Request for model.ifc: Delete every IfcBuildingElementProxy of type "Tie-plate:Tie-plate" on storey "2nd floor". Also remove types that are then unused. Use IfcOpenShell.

First a look at what the model holds.

```python
import ifcopenshell
import ifcopenshell.util.element

model = ifcopenshell.open("model.ifc")
print(model.schema)
storey = next(s for s in model.by_type("IfcBuildingStorey") if s.Name == "2nd floor")
proxies = [e for e in ifcopenshell.util.element.get_decomposition(storey) if e.is_a("IfcBuildingElementProxy")]
seen = {}
for e in proxies:
    element_type = ifcopenshell.util.element.get_type(e)
    name = element_type.Name if element_type not in (None, e) else None
    seen[name] = seen.get(name, 0) + 1
for name, count in sorted(seen.items(), key=str):
    print(count, "x", name)
```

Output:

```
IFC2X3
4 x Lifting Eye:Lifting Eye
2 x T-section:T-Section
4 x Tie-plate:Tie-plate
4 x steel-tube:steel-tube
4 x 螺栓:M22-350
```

```python
import ifcopenshell
import ifcopenshell.api.root
import ifcopenshell.util.element

model = ifcopenshell.open("model.ifc")

storey = next(s for s in model.by_type("IfcBuildingStorey") if s.Name == "2nd floor")
proxies = [e for e in ifcopenshell.util.element.get_decomposition(storey) if e.is_a("IfcBuildingElementProxy")]
targets = [e for e in proxies if (t := ifcopenshell.util.element.get_type(e)) not in (None, e) and t.Name == "Tie-plate:Tie-plate"]
types = {ifcopenshell.util.element.get_type(e) for e in targets} - {None, *targets}

for e in targets:
    ifcopenshell.api.root.remove_product(model, product=e)
print(len(targets), "removed")

unused = [t for t in types if not ifcopenshell.util.element.get_types(t)]
for t in unused:
    ifcopenshell.api.root.remove_product(model, product=t)
print(len(unused), "unused types removed")

model.write("model-out.ifc")
```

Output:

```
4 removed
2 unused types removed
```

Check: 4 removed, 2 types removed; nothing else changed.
